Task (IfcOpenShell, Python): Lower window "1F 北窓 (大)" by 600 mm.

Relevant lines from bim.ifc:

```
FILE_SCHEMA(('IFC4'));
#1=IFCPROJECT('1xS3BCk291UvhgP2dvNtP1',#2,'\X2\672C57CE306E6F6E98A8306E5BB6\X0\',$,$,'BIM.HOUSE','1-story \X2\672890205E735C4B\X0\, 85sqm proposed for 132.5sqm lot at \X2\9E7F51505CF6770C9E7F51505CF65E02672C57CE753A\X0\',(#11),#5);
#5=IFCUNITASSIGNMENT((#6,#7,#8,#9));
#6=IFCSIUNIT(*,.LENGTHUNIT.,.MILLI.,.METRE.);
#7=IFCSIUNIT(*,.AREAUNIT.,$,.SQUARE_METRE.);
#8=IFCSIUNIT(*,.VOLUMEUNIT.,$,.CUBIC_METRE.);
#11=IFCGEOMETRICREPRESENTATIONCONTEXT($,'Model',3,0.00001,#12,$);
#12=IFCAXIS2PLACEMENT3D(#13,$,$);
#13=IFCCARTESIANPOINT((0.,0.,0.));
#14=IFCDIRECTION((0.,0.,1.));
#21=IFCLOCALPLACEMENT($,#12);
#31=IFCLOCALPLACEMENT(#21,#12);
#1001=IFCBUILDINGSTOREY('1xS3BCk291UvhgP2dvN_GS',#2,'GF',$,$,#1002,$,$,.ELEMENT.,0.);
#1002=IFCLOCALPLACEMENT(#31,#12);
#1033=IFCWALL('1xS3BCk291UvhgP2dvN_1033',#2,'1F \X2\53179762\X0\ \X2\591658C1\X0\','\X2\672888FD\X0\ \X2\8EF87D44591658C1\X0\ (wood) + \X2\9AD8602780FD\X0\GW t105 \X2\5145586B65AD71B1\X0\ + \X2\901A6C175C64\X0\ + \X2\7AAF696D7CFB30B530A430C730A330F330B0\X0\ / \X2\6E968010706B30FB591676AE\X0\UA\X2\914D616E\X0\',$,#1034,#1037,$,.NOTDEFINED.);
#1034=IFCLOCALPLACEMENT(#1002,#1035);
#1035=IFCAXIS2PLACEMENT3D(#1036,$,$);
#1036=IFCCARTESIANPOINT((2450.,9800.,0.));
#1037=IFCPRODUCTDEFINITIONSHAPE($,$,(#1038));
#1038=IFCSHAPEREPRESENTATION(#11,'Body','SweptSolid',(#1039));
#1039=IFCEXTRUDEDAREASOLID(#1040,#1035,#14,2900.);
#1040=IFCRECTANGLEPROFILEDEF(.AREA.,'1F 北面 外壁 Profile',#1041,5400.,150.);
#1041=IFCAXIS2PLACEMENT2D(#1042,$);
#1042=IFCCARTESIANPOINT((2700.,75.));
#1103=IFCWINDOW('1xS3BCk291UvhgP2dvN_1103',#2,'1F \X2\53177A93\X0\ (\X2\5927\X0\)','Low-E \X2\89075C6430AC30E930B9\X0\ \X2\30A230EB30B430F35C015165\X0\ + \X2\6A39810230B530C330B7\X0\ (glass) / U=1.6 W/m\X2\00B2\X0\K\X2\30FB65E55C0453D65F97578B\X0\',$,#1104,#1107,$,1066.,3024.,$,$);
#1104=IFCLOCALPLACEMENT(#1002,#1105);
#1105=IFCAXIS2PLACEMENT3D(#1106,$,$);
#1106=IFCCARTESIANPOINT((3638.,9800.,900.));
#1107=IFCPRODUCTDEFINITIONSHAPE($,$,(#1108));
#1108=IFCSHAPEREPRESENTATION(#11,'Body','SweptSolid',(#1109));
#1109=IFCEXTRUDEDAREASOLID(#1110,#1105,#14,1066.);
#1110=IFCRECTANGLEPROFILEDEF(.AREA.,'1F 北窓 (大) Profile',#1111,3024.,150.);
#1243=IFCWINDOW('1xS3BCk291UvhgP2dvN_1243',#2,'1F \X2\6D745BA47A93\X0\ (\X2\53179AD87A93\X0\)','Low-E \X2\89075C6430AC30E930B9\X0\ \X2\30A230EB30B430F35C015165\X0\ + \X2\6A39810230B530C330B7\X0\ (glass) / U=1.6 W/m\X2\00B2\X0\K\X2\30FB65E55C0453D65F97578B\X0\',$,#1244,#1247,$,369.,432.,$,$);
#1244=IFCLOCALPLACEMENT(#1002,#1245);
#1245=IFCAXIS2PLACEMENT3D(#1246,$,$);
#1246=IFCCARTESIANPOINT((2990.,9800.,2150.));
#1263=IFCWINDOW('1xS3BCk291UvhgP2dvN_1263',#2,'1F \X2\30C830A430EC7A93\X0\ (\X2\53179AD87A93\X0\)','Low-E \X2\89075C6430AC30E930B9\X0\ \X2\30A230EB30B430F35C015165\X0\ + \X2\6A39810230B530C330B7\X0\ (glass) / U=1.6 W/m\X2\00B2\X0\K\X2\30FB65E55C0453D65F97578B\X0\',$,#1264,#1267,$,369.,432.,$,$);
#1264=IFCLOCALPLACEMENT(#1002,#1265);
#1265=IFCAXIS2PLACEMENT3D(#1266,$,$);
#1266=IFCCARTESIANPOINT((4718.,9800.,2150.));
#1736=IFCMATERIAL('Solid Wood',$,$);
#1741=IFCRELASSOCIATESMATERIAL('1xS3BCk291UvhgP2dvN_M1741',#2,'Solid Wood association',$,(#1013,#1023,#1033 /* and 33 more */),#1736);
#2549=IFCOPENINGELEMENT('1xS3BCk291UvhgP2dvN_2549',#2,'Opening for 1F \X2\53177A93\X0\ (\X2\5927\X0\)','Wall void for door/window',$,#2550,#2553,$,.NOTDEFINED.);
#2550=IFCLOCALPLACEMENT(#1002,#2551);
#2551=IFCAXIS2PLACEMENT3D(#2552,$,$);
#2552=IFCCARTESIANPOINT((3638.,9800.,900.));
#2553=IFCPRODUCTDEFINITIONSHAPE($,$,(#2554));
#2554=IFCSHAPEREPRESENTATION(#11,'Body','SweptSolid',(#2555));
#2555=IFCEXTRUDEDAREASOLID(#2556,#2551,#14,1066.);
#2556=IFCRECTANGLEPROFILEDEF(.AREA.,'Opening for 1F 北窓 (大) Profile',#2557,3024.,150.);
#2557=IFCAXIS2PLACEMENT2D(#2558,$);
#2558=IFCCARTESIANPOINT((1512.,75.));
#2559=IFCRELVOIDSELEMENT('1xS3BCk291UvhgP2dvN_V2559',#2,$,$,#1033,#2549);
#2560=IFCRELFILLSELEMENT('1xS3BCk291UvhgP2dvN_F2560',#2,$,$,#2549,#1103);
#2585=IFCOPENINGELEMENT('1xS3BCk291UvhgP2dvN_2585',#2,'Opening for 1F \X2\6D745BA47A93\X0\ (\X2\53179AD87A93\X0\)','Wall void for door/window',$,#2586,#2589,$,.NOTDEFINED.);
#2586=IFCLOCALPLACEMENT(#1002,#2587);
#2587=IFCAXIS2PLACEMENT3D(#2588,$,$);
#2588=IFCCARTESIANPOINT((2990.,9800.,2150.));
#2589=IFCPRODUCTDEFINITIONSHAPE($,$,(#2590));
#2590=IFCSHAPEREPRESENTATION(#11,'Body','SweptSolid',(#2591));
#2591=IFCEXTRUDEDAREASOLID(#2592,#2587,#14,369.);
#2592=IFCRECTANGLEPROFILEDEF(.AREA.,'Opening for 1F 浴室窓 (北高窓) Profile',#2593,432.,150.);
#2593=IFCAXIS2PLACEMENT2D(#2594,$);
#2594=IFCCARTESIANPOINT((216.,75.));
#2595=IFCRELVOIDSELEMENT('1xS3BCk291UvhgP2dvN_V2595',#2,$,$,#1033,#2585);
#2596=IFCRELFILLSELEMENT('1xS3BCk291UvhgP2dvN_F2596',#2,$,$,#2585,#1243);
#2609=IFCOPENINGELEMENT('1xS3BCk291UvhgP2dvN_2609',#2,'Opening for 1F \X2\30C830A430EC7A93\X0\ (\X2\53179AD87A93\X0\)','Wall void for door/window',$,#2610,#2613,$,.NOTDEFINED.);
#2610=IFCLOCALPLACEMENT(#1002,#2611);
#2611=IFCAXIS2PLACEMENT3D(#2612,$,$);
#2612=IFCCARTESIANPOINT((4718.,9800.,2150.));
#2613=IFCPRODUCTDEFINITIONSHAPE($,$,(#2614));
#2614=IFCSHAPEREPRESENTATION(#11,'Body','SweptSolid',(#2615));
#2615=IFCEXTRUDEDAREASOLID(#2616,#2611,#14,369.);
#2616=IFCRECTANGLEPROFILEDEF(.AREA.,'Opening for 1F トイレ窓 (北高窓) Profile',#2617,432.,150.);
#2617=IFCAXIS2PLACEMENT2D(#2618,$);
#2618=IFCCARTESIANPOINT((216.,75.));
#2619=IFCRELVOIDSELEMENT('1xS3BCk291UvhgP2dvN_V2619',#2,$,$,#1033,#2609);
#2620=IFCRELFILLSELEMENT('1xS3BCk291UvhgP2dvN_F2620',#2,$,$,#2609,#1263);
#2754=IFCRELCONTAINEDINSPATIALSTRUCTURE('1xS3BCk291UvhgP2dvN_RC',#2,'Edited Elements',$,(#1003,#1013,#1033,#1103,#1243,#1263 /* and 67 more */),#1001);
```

```python
import numpy as np
import ifcopenshell
import ifcopenshell.api.geometry
import ifcopenshell.util.placement
import ifcopenshell.util.unit

model = ifcopenshell.open("bim.ifc")
unit_scale = ifcopenshell.util.unit.calculate_unit_scale(model)

window = model.by_id(1103)
opening = window.FillsVoids[0].RelatingOpeningElement
dz = -600.0

shift = np.array([0.0, 0.0, dz])
# The window is not placed relative to its opening, so move both.
for product in (opening, window):
    matrix = ifcopenshell.util.placement.get_local_placement(product.ObjectPlacement)
    matrix[:3, 3] += shift
    ifcopenshell.api.geometry.edit_object_placement(model, product=product, matrix=matrix, is_si=False)

print(f"moved by {dz * unit_scale:+.3f} m")

model.write("bim_v2.ifc")
```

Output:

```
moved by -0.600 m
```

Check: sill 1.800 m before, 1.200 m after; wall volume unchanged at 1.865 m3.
